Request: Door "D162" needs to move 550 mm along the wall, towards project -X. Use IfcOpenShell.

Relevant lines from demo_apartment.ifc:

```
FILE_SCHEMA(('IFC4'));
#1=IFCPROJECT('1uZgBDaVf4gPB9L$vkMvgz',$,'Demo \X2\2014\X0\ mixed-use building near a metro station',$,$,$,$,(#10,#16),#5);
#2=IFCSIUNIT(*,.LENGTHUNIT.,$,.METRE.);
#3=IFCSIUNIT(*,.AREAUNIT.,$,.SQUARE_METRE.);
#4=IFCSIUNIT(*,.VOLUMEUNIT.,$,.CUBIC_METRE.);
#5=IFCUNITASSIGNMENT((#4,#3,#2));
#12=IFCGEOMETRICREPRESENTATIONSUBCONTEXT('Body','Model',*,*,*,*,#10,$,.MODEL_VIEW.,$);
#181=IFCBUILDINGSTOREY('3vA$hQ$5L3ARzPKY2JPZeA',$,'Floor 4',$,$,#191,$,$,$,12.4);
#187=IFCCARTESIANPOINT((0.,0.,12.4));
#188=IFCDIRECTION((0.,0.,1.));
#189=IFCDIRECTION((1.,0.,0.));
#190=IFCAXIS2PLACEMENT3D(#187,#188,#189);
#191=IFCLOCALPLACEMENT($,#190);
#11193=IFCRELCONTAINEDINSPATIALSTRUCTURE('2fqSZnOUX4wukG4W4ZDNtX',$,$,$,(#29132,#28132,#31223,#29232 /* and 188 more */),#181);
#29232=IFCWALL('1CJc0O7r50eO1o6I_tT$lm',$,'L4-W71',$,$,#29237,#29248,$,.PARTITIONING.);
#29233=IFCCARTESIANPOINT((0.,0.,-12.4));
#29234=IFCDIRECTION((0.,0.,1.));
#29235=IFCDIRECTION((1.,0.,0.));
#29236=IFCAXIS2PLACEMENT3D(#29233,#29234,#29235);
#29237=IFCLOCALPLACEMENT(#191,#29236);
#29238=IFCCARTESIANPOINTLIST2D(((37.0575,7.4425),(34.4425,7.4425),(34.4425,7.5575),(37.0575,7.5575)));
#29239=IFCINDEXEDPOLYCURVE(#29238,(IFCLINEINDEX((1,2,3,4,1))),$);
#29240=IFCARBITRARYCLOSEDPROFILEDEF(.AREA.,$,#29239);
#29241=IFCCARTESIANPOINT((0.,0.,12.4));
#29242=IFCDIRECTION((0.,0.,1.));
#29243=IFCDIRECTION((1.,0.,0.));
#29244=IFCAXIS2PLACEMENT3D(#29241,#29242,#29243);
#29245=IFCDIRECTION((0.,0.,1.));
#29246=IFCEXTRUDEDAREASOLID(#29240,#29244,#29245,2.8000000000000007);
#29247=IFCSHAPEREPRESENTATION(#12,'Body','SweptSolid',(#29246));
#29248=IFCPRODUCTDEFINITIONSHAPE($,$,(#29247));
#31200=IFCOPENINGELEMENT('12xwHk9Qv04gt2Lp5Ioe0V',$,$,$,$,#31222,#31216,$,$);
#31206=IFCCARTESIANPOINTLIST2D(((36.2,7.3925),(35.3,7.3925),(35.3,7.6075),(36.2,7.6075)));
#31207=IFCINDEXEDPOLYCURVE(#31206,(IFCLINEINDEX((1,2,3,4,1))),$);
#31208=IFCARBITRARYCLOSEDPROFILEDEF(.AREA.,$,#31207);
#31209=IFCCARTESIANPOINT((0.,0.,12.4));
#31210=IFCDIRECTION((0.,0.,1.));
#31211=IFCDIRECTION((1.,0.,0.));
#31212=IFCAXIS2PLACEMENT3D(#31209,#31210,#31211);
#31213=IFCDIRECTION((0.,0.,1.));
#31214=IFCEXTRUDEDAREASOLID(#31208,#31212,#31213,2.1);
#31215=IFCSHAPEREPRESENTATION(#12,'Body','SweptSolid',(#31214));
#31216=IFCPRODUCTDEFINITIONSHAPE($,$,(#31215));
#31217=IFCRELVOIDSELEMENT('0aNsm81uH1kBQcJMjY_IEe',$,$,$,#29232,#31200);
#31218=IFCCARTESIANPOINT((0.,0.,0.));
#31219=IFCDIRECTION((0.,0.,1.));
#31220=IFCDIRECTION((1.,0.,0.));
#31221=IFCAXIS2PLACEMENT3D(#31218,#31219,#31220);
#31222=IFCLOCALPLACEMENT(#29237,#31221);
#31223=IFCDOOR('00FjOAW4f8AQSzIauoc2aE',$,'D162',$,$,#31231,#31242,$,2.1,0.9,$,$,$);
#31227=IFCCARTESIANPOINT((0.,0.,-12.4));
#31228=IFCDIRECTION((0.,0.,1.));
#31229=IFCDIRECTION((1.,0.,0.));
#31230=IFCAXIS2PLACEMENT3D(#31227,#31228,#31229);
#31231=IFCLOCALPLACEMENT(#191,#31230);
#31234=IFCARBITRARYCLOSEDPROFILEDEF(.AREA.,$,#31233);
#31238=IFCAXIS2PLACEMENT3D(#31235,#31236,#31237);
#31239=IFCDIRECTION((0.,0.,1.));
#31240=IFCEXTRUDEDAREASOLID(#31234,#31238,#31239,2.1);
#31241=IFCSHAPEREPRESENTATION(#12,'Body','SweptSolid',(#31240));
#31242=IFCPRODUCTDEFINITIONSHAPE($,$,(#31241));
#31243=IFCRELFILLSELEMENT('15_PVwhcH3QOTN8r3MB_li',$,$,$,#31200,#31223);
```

```python
import ifcopenshell
import ifcopenshell.api.geometry
import ifcopenshell.util.placement

model = ifcopenshell.open("demo_apartment.ifc")

door = model.by_guid("00FjOAW4f8AQSzIauoc2aE")
opening = door.FillsVoids[0].RelatingOpeningElement
wall = opening.VoidsElements[0].RelatingBuildingElement

wall_matrix = ifcopenshell.util.placement.get_local_placement(wall.ObjectPlacement)
shift = wall_matrix[:3, 0] * -0.55
before = ifcopenshell.util.placement.get_local_placement(door.ObjectPlacement)[:3, 3].copy()

# The door is not placed relative to its opening, so move both.
for product in (opening, door):
    matrix = ifcopenshell.util.placement.get_local_placement(product.ObjectPlacement)
    matrix[:3, 3] += shift
    ifcopenshell.api.geometry.edit_object_placement(model, product=product, matrix=matrix, is_si=False)

after = ifcopenshell.util.placement.get_local_placement(door.ObjectPlacement)[:3, 3]
print("door moved by", (after - before).round(3) + 0.0)

model.write("demo_apartment_rev.ifc")
```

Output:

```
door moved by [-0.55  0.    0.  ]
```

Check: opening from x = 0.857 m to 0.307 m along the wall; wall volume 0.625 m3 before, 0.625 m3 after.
